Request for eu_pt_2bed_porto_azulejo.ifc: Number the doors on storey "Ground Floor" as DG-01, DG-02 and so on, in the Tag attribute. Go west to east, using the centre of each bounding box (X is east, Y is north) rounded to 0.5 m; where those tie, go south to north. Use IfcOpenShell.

First a look at what the model holds.

```python
import ifcopenshell
import ifcopenshell.util.element
import ifcopenshell.util.placement

model = ifcopenshell.open("eu_pt_2bed_porto_azulejo.ifc")
print(model.schema)
storey = next(s for s in model.by_type("IfcBuildingStorey") if s.Name == "Ground Floor")
doors = [e for e in ifcopenshell.util.element.get_decomposition(storey) if e.is_a("IfcDoor")]
for e in sorted(doors, key=lambda e: e.id()):
    origin = ifcopenshell.util.placement.get_local_placement(e.ObjectPlacement)[:3, 3]
    print(e.id(), e.Tag, e.Name, origin.round(2) + 0.0, sep=" | ")
```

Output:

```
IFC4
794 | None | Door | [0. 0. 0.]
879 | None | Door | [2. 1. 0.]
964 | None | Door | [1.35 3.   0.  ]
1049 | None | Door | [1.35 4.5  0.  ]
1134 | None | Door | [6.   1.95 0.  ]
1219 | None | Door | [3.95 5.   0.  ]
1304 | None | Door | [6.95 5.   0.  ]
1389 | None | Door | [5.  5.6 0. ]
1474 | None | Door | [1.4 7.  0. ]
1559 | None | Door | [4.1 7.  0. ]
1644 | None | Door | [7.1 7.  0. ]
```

```python
import ifcopenshell
import ifcopenshell.geom
import ifcopenshell.util.element
import ifcopenshell.util.shape

model = ifcopenshell.open("eu_pt_2bed_porto_azulejo.ifc")
settings = ifcopenshell.geom.settings()
settings.set("use-world-coords", True)


def centre(element):
    shape = ifcopenshell.geom.create_shape(settings, element)
    return ifcopenshell.util.shape.get_bbox_centroid(shape.geometry)


storey = next(s for s in model.by_type("IfcBuildingStorey") if s.Name == "Ground Floor")
doors = [e for e in ifcopenshell.util.element.get_decomposition(storey) if e.is_a("IfcDoor")]

# Insertion points can sit at a corner or the storey origin, so sort by the geometry (in metres).
centres = {e: centre(e) for e in doors}
doors.sort(key=lambda e: (round(centres[e][0] / 0.5), centres[e][1]))

for i, e in enumerate(doors, start=1):
    number = f"DG-{i:02d}"
    e.Tag = number
    print(e.id(), number)

model.write("eu_pt_2bed_porto_azulejo-out.ifc")
```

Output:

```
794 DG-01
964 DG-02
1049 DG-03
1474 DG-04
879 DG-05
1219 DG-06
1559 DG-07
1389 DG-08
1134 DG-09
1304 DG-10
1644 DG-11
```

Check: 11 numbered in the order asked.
